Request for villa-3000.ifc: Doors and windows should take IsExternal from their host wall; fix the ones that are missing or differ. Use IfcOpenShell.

First a look at what the model holds.

```python
import ifcopenshell
import ifcopenshell.util.element

model = ifcopenshell.open("villa-3000.ifc")
print(model.schema)
seen = {}
for e in model.by_type("IfcDoor") + model.by_type("IfcWindow"):
    if not e.FillsVoids:
        continue
    host = e.FillsVoids[0].RelatingOpeningElement.VoidsElements[0].RelatingBuildingElement
    own = ifcopenshell.util.element.get_pset(e, f"Pset_{e.is_a()[3:].removesuffix('StandardCase')}Common", "IsExternal")
    wall = ifcopenshell.util.element.get_pset(host, "Pset_WallCommon", "IsExternal")
    seen[e.is_a(), own, wall] = seen.get((e.is_a(), own, wall), 0) + 1
for (cls, own, wall), count in sorted(seen.items(), key=str):
    print(count, cls, "IsExternal:", own, "| host wall:", wall)
```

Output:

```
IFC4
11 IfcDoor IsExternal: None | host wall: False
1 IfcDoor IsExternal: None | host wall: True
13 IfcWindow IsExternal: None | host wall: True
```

```python
import ifcopenshell
import ifcopenshell.api.pset
import ifcopenshell.util.element

model = ifcopenshell.open("villa-3000.ifc")

count = 0
for ifc_class, pset_name in (("IfcDoor", "Pset_DoorCommon"), ("IfcWindow", "Pset_WindowCommon")):
    for e in model.by_type(ifc_class):
        if not e.FillsVoids:
            continue
        host = e.FillsVoids[0].RelatingOpeningElement.VoidsElements[0].RelatingBuildingElement
        external = ifcopenshell.util.element.get_pset(host, "Pset_WallCommon", "IsExternal")
        if external is None or ifcopenshell.util.element.get_pset(e, pset_name, "IsExternal") == external:
            continue
        pset = ifcopenshell.api.pset.add_pset(model, product=e, name=pset_name)
        ifcopenshell.api.pset.edit_pset(model, pset=pset, properties={"IsExternal": external})
        count += 1

print(count, "updated")

model.write("villa-3000_v2.ifc")
```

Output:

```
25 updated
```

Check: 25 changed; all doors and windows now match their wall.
